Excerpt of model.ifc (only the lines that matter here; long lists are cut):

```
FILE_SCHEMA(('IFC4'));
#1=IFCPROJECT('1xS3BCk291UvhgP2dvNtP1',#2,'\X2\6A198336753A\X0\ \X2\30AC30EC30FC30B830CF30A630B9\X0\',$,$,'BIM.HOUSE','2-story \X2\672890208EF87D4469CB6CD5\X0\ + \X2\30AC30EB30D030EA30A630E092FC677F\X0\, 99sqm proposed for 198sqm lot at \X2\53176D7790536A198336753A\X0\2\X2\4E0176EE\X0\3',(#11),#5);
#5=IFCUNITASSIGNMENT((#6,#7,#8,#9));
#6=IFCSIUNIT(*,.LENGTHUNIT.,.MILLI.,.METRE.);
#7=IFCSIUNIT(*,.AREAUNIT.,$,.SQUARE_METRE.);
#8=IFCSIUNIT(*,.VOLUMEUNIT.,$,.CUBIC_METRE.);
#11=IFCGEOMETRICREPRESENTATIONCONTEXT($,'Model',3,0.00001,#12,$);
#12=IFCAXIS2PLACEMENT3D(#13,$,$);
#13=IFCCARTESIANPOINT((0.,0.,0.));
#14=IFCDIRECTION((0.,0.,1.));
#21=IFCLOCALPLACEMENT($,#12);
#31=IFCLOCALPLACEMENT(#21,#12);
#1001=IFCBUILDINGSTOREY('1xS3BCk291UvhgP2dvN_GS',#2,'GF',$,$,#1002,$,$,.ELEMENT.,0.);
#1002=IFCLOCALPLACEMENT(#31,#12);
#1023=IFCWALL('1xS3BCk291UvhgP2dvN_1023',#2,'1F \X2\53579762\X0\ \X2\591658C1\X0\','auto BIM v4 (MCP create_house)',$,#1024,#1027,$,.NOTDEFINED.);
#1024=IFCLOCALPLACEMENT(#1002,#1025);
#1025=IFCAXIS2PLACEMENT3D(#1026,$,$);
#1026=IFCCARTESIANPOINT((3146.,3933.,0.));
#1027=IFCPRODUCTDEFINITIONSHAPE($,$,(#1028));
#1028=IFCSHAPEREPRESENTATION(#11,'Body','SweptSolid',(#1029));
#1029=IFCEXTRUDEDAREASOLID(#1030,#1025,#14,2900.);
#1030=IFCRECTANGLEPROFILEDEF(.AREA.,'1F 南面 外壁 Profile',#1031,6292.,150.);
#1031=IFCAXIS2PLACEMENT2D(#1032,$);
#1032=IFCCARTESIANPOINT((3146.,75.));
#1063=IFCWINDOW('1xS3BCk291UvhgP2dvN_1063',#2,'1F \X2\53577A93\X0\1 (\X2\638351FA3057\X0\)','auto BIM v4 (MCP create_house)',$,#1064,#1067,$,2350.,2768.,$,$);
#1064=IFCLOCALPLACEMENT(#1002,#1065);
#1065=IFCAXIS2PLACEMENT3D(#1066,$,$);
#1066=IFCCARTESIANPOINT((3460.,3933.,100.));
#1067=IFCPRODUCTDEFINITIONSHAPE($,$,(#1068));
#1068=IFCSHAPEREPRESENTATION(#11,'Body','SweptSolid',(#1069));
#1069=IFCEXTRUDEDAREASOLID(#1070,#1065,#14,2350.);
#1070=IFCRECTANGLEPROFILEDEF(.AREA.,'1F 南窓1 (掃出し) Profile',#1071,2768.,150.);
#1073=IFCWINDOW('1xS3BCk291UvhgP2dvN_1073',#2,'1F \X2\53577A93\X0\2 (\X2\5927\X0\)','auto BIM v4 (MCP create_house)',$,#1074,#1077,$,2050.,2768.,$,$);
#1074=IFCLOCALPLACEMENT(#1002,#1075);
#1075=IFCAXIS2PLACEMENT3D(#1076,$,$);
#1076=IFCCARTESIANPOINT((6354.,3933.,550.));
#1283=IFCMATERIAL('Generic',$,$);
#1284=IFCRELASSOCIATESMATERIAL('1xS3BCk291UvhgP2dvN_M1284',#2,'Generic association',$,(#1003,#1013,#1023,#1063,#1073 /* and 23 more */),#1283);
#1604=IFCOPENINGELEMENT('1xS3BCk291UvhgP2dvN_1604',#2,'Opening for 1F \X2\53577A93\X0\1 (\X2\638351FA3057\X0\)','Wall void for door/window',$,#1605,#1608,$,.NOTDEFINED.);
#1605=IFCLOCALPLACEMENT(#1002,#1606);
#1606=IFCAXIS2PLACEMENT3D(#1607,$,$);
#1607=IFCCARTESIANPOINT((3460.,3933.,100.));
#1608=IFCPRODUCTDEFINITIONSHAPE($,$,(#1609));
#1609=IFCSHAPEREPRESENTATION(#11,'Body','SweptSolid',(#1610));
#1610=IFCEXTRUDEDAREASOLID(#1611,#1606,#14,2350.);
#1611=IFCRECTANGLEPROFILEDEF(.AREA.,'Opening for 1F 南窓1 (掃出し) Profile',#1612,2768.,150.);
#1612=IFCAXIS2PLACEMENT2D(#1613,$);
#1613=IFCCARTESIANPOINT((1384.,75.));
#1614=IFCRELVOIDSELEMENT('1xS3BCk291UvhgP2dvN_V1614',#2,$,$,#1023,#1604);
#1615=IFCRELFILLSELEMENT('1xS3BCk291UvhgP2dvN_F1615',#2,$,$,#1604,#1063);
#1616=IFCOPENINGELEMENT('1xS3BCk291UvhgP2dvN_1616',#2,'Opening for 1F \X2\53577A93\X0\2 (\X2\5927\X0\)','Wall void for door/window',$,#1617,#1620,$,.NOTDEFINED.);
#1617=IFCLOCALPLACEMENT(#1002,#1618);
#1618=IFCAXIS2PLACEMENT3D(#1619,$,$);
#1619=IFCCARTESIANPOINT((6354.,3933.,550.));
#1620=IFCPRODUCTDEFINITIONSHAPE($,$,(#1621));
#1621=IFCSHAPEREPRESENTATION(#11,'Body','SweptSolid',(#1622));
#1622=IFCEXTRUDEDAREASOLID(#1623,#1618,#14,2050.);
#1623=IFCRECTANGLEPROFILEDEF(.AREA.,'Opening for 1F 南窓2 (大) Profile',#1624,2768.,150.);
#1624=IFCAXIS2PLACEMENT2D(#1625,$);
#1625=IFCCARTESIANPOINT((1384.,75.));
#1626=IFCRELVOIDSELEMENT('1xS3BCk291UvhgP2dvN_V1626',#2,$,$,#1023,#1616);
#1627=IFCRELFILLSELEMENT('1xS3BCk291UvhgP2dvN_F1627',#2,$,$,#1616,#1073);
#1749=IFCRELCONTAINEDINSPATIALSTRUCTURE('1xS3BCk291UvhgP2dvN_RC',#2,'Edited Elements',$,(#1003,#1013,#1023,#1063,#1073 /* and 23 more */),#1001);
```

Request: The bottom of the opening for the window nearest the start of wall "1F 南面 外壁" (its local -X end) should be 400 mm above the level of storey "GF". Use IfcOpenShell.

```python
import numpy as np
import ifcopenshell
import ifcopenshell.api.geometry
import ifcopenshell.geom
import ifcopenshell.util.element
import ifcopenshell.util.placement
import ifcopenshell.util.shape
import ifcopenshell.util.unit

model = ifcopenshell.open("model.ifc")
unit_scale = ifcopenshell.util.unit.calculate_unit_scale(model)

window = model.by_guid("1xS3BCk291UvhgP2dvN_1063")
opening = window.FillsVoids[0].RelatingOpeningElement
storey = ifcopenshell.util.element.get_container(window, ifc_class="IfcBuildingStorey")
level = ifcopenshell.util.placement.get_local_placement(storey.ObjectPlacement)[2, 3]

# The opening's origin need not be at the sill, so measure its lowest point.
shape = ifcopenshell.geom.create_shape(ifcopenshell.geom.settings(), opening)
bottom = ifcopenshell.util.shape.get_shape_bottom_elevation(shape, shape.geometry) / unit_scale
dz = level + 400.0 - bottom

shift = np.array([0.0, 0.0, dz])
# The window is not placed relative to its opening, so move both.
for product in (opening, window):
    matrix = ifcopenshell.util.placement.get_local_placement(product.ObjectPlacement)
    matrix[:3, 3] += shift
    ifcopenshell.api.geometry.edit_object_placement(model, product=product, matrix=matrix, is_si=False)

print(f"moved by {dz * unit_scale:+.3f} m")

model.write("model_edited.ifc")
```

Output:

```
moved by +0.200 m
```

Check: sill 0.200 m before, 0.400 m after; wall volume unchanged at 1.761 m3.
